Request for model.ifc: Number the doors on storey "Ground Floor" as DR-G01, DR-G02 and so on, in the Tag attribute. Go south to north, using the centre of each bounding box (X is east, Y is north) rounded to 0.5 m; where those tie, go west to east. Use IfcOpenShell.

First a look at what the model holds.

```python
import ifcopenshell
import ifcopenshell.util.element
import ifcopenshell.util.placement

model = ifcopenshell.open("model.ifc")
print(model.schema)
storey = next(s for s in model.by_type("IfcBuildingStorey") if s.Name == "Ground Floor")
doors = [e for e in ifcopenshell.util.element.get_decomposition(storey) if e.is_a("IfcDoor")]
for e in sorted(doors, key=lambda e: e.id()):
    origin = ifcopenshell.util.placement.get_local_placement(e.ObjectPlacement)[:3, 3]
    print(e.id(), e.Tag, e.Name, origin.round(2) + 0.0, sep=" | ")
```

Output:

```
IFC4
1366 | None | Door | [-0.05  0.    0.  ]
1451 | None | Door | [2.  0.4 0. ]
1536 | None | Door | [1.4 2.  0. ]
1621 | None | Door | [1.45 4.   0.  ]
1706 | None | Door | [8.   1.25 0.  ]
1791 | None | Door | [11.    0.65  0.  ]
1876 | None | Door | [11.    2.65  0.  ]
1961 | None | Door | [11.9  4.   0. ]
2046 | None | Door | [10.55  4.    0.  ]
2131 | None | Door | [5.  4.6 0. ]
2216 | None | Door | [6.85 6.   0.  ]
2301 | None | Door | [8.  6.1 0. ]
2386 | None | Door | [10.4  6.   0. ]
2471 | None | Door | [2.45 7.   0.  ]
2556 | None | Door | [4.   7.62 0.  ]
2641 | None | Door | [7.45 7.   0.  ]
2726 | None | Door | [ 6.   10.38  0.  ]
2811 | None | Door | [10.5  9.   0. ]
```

```python
import ifcopenshell
import ifcopenshell.geom
import ifcopenshell.util.element
import ifcopenshell.util.shape

model = ifcopenshell.open("model.ifc")
settings = ifcopenshell.geom.settings()
settings.set("use-world-coords", True)


def centre(element):
    shape = ifcopenshell.geom.create_shape(settings, element)
    return ifcopenshell.util.shape.get_bbox_centroid(shape.geometry)


storey = next(s for s in model.by_type("IfcBuildingStorey") if s.Name == "Ground Floor")
doors = [e for e in ifcopenshell.util.element.get_decomposition(storey) if e.is_a("IfcDoor")]

# Insertion points can sit at a corner or the storey origin, so sort by the geometry (in metres).
centres = {e: centre(e) for e in doors}
doors.sort(key=lambda e: (round(centres[e][1] / 0.5), centres[e][0]))

for i, e in enumerate(doors, start=1):
    number = f"DR-G{i:02d}"
    e.Tag = number
    print(e.id(), number)

model.write("model_v2.ifc")
```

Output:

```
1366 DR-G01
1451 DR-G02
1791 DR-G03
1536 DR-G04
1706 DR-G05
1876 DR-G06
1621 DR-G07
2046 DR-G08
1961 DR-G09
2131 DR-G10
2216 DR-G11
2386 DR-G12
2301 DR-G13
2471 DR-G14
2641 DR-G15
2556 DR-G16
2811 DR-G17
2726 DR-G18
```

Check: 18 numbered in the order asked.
